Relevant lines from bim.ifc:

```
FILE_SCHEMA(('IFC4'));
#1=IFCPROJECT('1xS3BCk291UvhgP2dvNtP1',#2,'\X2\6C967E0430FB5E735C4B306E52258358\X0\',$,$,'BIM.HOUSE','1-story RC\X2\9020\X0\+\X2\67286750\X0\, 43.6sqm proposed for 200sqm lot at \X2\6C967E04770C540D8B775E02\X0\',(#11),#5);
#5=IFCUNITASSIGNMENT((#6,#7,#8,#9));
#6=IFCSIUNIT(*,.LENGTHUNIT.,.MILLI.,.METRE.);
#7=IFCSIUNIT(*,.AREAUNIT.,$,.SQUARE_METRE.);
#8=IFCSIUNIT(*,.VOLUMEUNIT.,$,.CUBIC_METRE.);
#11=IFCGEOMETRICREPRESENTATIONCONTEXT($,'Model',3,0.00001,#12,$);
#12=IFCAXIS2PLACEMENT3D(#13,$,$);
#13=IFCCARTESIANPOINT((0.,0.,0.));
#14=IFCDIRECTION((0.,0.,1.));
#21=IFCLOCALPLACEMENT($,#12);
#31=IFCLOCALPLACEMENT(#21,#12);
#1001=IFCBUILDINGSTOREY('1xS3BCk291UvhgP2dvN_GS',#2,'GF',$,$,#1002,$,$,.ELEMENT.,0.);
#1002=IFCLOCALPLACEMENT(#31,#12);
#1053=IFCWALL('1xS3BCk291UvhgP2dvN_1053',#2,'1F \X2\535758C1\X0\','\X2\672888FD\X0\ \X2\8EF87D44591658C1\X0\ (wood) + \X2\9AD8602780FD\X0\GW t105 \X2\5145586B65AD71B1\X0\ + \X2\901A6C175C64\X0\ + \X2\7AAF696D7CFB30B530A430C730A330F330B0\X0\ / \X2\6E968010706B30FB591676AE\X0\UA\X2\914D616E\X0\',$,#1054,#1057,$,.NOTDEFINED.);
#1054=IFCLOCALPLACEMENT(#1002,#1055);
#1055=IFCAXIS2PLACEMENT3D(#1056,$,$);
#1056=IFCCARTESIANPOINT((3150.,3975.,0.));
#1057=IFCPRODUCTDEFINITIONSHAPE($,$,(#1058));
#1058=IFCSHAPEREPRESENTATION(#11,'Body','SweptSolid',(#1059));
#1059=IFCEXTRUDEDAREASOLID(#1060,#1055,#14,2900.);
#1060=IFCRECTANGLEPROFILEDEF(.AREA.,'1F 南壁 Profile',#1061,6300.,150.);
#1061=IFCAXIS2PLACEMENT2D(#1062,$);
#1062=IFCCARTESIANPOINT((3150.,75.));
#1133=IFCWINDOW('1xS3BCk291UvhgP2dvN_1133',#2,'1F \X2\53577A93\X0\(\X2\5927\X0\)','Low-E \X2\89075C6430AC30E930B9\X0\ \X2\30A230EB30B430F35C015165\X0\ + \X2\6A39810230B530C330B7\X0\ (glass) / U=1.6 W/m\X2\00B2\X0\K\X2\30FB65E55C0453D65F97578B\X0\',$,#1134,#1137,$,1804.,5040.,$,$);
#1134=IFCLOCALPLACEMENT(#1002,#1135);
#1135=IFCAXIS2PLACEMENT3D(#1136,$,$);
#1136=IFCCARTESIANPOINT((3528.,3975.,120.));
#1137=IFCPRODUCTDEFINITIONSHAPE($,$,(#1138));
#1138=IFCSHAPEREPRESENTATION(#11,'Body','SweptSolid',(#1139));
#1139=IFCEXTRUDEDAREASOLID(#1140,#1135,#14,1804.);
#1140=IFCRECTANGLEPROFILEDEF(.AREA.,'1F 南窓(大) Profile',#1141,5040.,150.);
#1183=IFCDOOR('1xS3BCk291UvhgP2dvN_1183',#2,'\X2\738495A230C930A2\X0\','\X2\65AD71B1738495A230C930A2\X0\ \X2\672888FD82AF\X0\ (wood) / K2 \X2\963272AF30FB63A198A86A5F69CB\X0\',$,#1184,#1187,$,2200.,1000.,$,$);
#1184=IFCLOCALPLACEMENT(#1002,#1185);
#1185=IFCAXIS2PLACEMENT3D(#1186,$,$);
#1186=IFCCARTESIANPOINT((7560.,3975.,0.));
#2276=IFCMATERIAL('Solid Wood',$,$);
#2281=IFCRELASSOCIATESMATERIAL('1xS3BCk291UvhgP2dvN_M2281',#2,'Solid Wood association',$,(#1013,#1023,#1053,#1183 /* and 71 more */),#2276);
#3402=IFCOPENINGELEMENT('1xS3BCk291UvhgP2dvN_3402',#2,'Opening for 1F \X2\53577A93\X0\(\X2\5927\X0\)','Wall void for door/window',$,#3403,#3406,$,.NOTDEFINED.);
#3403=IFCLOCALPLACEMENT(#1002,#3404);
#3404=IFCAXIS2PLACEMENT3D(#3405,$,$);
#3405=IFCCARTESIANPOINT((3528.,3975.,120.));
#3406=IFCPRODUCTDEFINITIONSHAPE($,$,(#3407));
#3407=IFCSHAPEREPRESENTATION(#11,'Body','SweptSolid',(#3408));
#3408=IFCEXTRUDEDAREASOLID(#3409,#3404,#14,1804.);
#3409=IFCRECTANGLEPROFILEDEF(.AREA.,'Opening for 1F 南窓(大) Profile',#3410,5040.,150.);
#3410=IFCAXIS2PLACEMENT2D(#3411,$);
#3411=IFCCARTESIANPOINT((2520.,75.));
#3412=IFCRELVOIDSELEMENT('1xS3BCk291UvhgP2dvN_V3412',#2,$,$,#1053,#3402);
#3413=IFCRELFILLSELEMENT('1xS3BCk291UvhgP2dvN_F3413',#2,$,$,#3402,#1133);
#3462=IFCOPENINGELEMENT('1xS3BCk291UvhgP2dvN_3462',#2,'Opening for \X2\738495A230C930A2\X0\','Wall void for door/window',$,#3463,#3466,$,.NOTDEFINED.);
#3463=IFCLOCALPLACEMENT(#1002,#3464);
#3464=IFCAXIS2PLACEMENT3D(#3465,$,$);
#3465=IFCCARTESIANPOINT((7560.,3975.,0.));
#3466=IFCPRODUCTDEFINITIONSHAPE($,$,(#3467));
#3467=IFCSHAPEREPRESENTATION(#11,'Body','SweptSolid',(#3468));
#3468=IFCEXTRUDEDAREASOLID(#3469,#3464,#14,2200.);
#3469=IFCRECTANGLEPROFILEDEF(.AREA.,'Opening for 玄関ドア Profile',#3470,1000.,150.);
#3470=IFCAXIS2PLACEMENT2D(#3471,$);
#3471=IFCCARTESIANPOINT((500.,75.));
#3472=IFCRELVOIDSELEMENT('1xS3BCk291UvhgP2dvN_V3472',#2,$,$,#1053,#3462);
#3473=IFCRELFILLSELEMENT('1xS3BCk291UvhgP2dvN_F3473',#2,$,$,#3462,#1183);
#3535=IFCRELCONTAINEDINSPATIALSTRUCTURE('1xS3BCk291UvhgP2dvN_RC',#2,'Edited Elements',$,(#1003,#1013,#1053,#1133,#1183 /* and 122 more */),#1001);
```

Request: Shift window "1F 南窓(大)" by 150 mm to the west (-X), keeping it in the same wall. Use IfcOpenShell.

```python
import ifcopenshell
import ifcopenshell.api.geometry
import ifcopenshell.util.placement
import ifcopenshell.util.unit

model = ifcopenshell.open("bim.ifc")
unit_scale = ifcopenshell.util.unit.calculate_unit_scale(model)

window = model.by_guid("1xS3BCk291UvhgP2dvN_1133")
opening = window.FillsVoids[0].RelatingOpeningElement
wall = opening.VoidsElements[0].RelatingBuildingElement

wall_matrix = ifcopenshell.util.placement.get_local_placement(wall.ObjectPlacement)
shift = wall_matrix[:3, 0] * -0.15 / unit_scale
before = ifcopenshell.util.placement.get_local_placement(window.ObjectPlacement)[:3, 3].copy()

# The window is not placed relative to its opening, so move both.
for product in (opening, window):
    matrix = ifcopenshell.util.placement.get_local_placement(product.ObjectPlacement)
    matrix[:3, 3] += shift
    ifcopenshell.api.geometry.edit_object_placement(model, product=product, matrix=matrix, is_si=False)

after = ifcopenshell.util.placement.get_local_placement(window.ObjectPlacement)[:3, 3]
print("window moved by", (after - before).round(3) + 0.0)

model.write("bim_rev.ifc")
```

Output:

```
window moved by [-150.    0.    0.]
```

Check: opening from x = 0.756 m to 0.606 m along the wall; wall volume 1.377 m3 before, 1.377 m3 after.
